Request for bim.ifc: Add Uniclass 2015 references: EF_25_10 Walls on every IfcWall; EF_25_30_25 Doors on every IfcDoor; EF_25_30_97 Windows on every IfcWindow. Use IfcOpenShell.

First a look at what the model holds.

```python
import ifcopenshell

model = ifcopenshell.open("bim.ifc")
print(model.schema)
print("classifications:", [c.Name for c in model.by_type("IfcClassification")])
for ifc_class in ("IfcDoor", "IfcRoof", "IfcStair", "IfcWall", "IfcWindow"):
    print(ifc_class, len(model.by_type(ifc_class)))
```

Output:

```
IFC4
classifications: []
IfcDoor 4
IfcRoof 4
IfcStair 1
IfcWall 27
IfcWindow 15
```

```python
import ifcopenshell
import ifcopenshell.api.classification

model = ifcopenshell.open("bim.ifc")

system = ifcopenshell.api.classification.add_classification(model, classification="Uniclass 2015")

codes = {
    "IfcWall": ("EF_25_10", "Walls"),
    "IfcDoor": ("EF_25_30_25", "Doors"),
    "IfcWindow": ("EF_25_30_97", "Windows"),
}
for ifc_class, (code, name) in codes.items():
    products = model.by_type(ifc_class)
    ifcopenshell.api.classification.add_reference(
        model, products=products, classification=system, identification=code, name=name
    )
    print(code, len(products))

model.write("bim-out.ifc")
```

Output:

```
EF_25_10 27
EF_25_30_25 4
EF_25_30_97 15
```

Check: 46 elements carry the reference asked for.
